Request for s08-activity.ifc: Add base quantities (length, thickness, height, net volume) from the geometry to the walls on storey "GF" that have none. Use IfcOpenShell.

First a look at what the model holds.

```python
import ifcopenshell
import ifcopenshell.util.element
import ifcopenshell.util.unit

model = ifcopenshell.open("s08-activity.ifc")
print(model.schema)
for unit_type in ("LENGTHUNIT", "AREAUNIT", "VOLUMEUNIT"):
    print(unit_type, ifcopenshell.util.unit.calculate_unit_scale(model, unit_type))
storey = next(s for s in model.by_type("IfcBuildingStorey") if s.Name == "GF")
walls = [e for e in ifcopenshell.util.element.get_decomposition(storey) if e.is_a("IfcWall")]
for e in sorted(walls, key=lambda e: e.id()):
    print(e.id(), e.is_a(), e.Name, list(ifcopenshell.util.element.get_psets(e, qtos_only=True)), sep=" | ")
```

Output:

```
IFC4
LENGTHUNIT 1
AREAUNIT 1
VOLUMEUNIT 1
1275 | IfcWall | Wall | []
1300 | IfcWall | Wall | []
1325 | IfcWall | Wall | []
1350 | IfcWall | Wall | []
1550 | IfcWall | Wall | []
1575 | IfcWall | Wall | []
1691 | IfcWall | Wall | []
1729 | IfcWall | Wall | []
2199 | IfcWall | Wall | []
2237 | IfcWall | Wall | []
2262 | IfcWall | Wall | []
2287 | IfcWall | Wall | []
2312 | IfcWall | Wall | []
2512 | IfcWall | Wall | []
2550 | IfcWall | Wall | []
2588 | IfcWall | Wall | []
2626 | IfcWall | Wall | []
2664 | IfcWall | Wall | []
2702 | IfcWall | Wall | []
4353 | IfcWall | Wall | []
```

```python
import ifcopenshell
import ifcopenshell.api.pset
import ifcopenshell.geom
import ifcopenshell.util.element
import ifcopenshell.util.shape
import ifcopenshell.util.unit

model = ifcopenshell.open("s08-activity.ifc")
unit_scale = ifcopenshell.util.unit.calculate_unit_scale(model)
volume_scale = ifcopenshell.util.unit.calculate_unit_scale(model, "VOLUMEUNIT")
settings = ifcopenshell.geom.settings()

storey = next(s for s in model.by_type("IfcBuildingStorey") if s.Name == "GF")
walls = [e for e in ifcopenshell.util.element.get_decomposition(storey) if e.is_a("IfcWall")]

for e in sorted(walls, key=lambda e: e.id()):
    if ifcopenshell.util.element.get_psets(e, qtos_only=True, should_inherit=False):
        continue
    # Geometry comes back in metres, in the element's own axes.
    shape = ifcopenshell.geom.create_shape(settings, e)
    values = {
        "Length": ifcopenshell.util.shape.get_x(shape.geometry) / unit_scale,
        "Width": ifcopenshell.util.shape.get_y(shape.geometry) / unit_scale,
        "Height": ifcopenshell.util.shape.get_z(shape.geometry) / unit_scale,
        "NetVolume": ifcopenshell.util.shape.get_volume(shape.geometry) / volume_scale,
    }
    qto = ifcopenshell.api.pset.add_qto(model, product=e, name="Qto_WallBaseQuantities")
    ifcopenshell.api.pset.edit_qto(model, qto=qto, properties=values)
    print(e.id(), {k: round(v, 3) for k, v in values.items()})

model.write("s08-activity-out.ifc")
```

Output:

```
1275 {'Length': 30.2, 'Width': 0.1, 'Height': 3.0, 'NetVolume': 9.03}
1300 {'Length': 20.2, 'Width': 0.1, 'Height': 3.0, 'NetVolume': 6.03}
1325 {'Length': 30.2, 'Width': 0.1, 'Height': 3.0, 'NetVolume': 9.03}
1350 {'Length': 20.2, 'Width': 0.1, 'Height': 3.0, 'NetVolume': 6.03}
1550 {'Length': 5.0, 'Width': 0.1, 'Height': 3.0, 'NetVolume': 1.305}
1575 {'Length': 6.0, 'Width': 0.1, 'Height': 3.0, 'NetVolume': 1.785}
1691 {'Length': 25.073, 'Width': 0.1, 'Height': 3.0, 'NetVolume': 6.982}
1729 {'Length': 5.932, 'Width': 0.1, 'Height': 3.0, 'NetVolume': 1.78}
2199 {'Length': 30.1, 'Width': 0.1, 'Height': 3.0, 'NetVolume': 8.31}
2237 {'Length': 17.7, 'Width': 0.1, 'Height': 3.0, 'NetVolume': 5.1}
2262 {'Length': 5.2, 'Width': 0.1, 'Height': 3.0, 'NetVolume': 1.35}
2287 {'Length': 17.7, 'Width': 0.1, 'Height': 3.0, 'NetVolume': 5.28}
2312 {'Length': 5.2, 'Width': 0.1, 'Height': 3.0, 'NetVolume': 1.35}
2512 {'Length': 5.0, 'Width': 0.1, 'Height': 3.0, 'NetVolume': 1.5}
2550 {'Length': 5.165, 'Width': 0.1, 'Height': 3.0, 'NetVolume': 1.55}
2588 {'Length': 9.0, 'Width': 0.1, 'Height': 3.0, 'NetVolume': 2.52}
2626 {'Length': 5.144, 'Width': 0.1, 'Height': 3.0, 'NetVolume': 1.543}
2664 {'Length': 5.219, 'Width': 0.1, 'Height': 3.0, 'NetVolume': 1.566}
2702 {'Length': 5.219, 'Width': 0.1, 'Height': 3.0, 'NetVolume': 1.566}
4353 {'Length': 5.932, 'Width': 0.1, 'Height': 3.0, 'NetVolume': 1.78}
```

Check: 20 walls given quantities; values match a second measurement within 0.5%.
